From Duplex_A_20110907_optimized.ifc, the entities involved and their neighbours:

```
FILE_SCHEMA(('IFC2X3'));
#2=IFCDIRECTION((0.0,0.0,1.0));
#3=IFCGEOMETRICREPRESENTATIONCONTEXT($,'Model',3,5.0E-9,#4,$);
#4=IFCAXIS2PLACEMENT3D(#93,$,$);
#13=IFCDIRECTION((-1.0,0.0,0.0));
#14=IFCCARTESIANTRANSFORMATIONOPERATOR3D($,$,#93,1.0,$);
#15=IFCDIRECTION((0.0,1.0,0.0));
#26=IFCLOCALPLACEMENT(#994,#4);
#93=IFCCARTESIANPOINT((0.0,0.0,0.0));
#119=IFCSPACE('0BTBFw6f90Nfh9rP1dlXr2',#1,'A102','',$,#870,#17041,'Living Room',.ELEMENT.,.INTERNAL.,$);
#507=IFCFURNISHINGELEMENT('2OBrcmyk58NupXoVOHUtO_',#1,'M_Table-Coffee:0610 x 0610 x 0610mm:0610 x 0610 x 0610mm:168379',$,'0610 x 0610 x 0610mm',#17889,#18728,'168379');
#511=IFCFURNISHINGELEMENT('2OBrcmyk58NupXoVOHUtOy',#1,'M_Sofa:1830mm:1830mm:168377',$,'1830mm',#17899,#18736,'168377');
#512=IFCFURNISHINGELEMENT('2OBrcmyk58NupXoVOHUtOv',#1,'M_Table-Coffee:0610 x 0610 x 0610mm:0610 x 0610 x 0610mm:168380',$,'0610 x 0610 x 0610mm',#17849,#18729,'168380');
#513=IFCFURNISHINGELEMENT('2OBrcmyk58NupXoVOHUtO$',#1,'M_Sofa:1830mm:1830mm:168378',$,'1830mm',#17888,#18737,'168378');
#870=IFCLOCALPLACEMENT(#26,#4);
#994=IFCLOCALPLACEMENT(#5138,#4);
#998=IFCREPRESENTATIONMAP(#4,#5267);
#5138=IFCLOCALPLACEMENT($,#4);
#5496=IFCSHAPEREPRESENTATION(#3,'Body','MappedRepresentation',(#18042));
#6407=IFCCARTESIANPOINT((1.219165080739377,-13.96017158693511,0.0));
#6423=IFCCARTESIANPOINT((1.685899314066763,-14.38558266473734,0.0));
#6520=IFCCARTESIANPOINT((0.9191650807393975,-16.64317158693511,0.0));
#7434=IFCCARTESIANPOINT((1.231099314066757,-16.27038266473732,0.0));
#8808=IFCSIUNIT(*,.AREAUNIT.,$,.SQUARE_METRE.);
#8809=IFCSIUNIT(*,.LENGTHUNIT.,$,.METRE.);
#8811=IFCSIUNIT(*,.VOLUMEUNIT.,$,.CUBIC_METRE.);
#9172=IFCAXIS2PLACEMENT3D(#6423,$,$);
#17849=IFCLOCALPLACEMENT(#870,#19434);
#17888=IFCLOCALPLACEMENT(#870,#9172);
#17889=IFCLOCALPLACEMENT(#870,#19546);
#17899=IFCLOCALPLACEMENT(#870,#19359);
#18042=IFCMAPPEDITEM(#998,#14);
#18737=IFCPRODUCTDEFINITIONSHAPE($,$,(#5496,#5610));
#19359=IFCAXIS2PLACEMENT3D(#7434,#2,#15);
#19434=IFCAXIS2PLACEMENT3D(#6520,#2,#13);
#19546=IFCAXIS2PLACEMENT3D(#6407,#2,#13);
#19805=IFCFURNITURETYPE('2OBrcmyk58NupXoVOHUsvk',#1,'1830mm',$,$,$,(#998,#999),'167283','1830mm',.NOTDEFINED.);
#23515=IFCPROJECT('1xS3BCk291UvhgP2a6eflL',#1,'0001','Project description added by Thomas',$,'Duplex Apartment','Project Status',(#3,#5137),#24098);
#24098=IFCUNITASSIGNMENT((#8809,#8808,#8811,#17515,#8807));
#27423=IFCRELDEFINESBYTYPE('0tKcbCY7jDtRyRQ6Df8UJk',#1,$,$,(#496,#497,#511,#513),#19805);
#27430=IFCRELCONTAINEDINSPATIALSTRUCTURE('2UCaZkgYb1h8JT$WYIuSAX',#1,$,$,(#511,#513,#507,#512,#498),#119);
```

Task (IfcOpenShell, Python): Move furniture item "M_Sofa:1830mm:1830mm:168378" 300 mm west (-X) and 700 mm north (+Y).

```python
import ifcopenshell
import ifcopenshell.api.geometry
import ifcopenshell.util.placement
import ifcopenshell.util.unit

model = ifcopenshell.open("Duplex_A_20110907_optimized.ifc")
unit_scale = ifcopenshell.util.unit.calculate_unit_scale(model)

item = model.by_guid("2OBrcmyk58NupXoVOHUtO$")
matrix = ifcopenshell.util.placement.get_local_placement(item.ObjectPlacement)
matrix[0, 3] -= 0.3 / unit_scale
matrix[1, 3] += 0.7 / unit_scale
ifcopenshell.api.geometry.edit_object_placement(model, product=item, matrix=matrix, is_si=False)

print(ifcopenshell.util.placement.get_local_placement(item.ObjectPlacement).round(3) + 0.0)

model.write("Duplex_A_20110907_optimized_edited.ifc")
```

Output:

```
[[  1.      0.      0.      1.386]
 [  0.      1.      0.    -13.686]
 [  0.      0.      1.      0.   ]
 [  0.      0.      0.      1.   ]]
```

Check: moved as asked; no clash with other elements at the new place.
